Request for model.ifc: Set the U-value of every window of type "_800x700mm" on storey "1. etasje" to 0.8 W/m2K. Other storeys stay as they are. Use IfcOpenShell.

First a look at what the model holds.

```python
import ifcopenshell
import ifcopenshell.util.element

model = ifcopenshell.open("model.ifc")
print(model.schema)
storey = next(s for s in model.by_type("IfcBuildingStorey") if s.Name == "1. etasje")
windows = [e for e in ifcopenshell.util.element.get_decomposition(storey) if e.is_a("IfcWindow")]
seen = {}
for e in windows:
    element_type = ifcopenshell.util.element.get_type(e)
    key = (element_type.Name if element_type != e and element_type else None, ifcopenshell.util.element.get_pset(e, "Pset_WindowCommon", "ThermalTransmittance"))
    seen[key] = seen.get(key, 0) + 1
for (name, value), count in sorted(seen.items(), key=str):
    print(count, "x", name, "|", value)
```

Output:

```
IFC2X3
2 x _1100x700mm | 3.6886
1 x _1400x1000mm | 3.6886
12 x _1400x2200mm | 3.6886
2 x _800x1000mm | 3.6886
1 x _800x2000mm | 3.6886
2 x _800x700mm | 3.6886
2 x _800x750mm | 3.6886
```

```python
import ifcopenshell
import ifcopenshell.api.pset
import ifcopenshell.util.element

model = ifcopenshell.open("model.ifc")

storey = next(s for s in model.by_type("IfcBuildingStorey") if s.Name == "1. etasje")
windows = [e for e in ifcopenshell.util.element.get_decomposition(storey) if e.is_a("IfcWindow")]

count = 0
for e in windows:
    element_type = ifcopenshell.util.element.get_type(e)
    if element_type in (None, e) or element_type.Name != "_800x700mm":
        continue
    # add_pset returns the element's existing set when there is one.
    pset = ifcopenshell.api.pset.add_pset(model, product=e, name="Pset_WindowCommon")
    ifcopenshell.api.pset.edit_pset(model, pset=pset, properties={"ThermalTransmittance": 0.8})
    count += 1

print(count, "windows updated")

model.write("model-out.ifc")
```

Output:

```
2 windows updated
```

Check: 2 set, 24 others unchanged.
